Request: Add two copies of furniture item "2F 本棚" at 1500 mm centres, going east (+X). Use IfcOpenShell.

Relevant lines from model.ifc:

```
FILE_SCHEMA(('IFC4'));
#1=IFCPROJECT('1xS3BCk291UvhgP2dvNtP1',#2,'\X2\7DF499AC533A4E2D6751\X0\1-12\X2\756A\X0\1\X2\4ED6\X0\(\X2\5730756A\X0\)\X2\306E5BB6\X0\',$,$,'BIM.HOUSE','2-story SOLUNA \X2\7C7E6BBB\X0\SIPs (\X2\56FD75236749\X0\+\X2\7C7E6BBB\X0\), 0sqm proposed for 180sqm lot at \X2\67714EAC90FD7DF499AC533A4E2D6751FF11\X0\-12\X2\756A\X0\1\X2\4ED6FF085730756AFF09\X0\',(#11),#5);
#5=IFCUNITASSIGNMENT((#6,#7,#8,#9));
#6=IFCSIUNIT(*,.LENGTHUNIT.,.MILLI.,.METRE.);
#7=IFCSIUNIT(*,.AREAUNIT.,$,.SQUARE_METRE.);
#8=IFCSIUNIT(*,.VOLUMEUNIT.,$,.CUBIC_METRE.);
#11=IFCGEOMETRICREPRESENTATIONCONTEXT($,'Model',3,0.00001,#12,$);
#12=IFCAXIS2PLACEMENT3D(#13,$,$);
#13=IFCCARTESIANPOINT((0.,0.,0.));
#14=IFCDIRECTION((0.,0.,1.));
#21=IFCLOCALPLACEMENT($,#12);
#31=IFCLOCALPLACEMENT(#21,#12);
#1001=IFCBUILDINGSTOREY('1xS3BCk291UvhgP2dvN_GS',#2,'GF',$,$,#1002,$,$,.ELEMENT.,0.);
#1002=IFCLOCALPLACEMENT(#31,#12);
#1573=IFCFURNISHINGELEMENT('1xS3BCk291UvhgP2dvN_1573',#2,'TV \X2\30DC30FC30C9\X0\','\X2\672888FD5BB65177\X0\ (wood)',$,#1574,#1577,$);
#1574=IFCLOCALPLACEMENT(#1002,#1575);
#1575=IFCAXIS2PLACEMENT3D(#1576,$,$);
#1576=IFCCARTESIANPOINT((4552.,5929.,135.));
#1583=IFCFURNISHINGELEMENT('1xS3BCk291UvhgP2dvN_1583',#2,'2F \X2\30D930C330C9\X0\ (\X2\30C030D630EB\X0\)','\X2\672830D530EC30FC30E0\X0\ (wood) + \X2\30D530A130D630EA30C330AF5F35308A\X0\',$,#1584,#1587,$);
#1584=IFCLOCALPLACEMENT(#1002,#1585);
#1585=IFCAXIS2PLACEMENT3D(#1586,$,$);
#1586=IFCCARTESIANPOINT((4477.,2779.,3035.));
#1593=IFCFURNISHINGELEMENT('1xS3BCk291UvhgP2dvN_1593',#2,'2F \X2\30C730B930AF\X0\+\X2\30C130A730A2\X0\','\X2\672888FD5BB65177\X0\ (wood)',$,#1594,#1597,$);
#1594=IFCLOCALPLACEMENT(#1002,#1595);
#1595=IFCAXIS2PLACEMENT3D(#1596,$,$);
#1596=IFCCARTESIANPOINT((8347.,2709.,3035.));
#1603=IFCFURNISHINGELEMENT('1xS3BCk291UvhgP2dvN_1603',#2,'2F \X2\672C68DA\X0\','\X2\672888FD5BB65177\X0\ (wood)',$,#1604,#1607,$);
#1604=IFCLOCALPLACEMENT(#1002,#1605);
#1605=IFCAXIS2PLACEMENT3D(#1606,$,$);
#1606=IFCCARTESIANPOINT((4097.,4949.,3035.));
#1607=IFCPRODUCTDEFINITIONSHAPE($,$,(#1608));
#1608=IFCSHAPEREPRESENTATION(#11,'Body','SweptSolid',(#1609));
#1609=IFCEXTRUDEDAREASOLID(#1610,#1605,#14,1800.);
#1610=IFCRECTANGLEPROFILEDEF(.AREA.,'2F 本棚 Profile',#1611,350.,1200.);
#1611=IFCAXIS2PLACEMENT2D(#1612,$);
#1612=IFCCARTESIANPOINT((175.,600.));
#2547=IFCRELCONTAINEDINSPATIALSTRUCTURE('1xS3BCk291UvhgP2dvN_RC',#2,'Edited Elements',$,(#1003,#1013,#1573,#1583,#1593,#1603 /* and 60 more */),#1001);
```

```python
import numpy as np
import ifcopenshell
import ifcopenshell.api.geometry
import ifcopenshell.api.root
import ifcopenshell.util.element
import ifcopenshell.util.placement

model = ifcopenshell.open("model.ifc")


def reuse_history(source, copy):
    """copy_class also copies each property set's owner history, people and application; keep the originals."""
    for rel in copy.IsDefinedBy:
        if rel.is_a("IfcRelDefinesByProperties") and (history := rel.RelatingPropertyDefinition.OwnerHistory):
            rel.RelatingPropertyDefinition.OwnerHistory = source.OwnerHistory
            ifcopenshell.util.element.remove_deep2(model, history)


source = model.by_id(1603)
base = ifcopenshell.util.placement.get_local_placement(source.ObjectPlacement)
step = np.array([1.0, 0.0, 0.0]) * 1500.0

for i in range(1, 3):
    copy = ifcopenshell.api.root.copy_class(model, product=source)
    copy.Representation = ifcopenshell.util.element.copy_deep(
        model, source.Representation, exclude=["IfcGeometricRepresentationContext", "IfcRepresentationMap"]
    )
    reuse_history(source, copy)
    matrix = base.copy()
    matrix[:3, 3] += i * step
    print("added at", matrix[:3, 3].round(3) + 0.0)
    ifcopenshell.api.geometry.edit_object_placement(model, product=copy, matrix=matrix, is_si=False)

model.write("model_updated.ifc")
```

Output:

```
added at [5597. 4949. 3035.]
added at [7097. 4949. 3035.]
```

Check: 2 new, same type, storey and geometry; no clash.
